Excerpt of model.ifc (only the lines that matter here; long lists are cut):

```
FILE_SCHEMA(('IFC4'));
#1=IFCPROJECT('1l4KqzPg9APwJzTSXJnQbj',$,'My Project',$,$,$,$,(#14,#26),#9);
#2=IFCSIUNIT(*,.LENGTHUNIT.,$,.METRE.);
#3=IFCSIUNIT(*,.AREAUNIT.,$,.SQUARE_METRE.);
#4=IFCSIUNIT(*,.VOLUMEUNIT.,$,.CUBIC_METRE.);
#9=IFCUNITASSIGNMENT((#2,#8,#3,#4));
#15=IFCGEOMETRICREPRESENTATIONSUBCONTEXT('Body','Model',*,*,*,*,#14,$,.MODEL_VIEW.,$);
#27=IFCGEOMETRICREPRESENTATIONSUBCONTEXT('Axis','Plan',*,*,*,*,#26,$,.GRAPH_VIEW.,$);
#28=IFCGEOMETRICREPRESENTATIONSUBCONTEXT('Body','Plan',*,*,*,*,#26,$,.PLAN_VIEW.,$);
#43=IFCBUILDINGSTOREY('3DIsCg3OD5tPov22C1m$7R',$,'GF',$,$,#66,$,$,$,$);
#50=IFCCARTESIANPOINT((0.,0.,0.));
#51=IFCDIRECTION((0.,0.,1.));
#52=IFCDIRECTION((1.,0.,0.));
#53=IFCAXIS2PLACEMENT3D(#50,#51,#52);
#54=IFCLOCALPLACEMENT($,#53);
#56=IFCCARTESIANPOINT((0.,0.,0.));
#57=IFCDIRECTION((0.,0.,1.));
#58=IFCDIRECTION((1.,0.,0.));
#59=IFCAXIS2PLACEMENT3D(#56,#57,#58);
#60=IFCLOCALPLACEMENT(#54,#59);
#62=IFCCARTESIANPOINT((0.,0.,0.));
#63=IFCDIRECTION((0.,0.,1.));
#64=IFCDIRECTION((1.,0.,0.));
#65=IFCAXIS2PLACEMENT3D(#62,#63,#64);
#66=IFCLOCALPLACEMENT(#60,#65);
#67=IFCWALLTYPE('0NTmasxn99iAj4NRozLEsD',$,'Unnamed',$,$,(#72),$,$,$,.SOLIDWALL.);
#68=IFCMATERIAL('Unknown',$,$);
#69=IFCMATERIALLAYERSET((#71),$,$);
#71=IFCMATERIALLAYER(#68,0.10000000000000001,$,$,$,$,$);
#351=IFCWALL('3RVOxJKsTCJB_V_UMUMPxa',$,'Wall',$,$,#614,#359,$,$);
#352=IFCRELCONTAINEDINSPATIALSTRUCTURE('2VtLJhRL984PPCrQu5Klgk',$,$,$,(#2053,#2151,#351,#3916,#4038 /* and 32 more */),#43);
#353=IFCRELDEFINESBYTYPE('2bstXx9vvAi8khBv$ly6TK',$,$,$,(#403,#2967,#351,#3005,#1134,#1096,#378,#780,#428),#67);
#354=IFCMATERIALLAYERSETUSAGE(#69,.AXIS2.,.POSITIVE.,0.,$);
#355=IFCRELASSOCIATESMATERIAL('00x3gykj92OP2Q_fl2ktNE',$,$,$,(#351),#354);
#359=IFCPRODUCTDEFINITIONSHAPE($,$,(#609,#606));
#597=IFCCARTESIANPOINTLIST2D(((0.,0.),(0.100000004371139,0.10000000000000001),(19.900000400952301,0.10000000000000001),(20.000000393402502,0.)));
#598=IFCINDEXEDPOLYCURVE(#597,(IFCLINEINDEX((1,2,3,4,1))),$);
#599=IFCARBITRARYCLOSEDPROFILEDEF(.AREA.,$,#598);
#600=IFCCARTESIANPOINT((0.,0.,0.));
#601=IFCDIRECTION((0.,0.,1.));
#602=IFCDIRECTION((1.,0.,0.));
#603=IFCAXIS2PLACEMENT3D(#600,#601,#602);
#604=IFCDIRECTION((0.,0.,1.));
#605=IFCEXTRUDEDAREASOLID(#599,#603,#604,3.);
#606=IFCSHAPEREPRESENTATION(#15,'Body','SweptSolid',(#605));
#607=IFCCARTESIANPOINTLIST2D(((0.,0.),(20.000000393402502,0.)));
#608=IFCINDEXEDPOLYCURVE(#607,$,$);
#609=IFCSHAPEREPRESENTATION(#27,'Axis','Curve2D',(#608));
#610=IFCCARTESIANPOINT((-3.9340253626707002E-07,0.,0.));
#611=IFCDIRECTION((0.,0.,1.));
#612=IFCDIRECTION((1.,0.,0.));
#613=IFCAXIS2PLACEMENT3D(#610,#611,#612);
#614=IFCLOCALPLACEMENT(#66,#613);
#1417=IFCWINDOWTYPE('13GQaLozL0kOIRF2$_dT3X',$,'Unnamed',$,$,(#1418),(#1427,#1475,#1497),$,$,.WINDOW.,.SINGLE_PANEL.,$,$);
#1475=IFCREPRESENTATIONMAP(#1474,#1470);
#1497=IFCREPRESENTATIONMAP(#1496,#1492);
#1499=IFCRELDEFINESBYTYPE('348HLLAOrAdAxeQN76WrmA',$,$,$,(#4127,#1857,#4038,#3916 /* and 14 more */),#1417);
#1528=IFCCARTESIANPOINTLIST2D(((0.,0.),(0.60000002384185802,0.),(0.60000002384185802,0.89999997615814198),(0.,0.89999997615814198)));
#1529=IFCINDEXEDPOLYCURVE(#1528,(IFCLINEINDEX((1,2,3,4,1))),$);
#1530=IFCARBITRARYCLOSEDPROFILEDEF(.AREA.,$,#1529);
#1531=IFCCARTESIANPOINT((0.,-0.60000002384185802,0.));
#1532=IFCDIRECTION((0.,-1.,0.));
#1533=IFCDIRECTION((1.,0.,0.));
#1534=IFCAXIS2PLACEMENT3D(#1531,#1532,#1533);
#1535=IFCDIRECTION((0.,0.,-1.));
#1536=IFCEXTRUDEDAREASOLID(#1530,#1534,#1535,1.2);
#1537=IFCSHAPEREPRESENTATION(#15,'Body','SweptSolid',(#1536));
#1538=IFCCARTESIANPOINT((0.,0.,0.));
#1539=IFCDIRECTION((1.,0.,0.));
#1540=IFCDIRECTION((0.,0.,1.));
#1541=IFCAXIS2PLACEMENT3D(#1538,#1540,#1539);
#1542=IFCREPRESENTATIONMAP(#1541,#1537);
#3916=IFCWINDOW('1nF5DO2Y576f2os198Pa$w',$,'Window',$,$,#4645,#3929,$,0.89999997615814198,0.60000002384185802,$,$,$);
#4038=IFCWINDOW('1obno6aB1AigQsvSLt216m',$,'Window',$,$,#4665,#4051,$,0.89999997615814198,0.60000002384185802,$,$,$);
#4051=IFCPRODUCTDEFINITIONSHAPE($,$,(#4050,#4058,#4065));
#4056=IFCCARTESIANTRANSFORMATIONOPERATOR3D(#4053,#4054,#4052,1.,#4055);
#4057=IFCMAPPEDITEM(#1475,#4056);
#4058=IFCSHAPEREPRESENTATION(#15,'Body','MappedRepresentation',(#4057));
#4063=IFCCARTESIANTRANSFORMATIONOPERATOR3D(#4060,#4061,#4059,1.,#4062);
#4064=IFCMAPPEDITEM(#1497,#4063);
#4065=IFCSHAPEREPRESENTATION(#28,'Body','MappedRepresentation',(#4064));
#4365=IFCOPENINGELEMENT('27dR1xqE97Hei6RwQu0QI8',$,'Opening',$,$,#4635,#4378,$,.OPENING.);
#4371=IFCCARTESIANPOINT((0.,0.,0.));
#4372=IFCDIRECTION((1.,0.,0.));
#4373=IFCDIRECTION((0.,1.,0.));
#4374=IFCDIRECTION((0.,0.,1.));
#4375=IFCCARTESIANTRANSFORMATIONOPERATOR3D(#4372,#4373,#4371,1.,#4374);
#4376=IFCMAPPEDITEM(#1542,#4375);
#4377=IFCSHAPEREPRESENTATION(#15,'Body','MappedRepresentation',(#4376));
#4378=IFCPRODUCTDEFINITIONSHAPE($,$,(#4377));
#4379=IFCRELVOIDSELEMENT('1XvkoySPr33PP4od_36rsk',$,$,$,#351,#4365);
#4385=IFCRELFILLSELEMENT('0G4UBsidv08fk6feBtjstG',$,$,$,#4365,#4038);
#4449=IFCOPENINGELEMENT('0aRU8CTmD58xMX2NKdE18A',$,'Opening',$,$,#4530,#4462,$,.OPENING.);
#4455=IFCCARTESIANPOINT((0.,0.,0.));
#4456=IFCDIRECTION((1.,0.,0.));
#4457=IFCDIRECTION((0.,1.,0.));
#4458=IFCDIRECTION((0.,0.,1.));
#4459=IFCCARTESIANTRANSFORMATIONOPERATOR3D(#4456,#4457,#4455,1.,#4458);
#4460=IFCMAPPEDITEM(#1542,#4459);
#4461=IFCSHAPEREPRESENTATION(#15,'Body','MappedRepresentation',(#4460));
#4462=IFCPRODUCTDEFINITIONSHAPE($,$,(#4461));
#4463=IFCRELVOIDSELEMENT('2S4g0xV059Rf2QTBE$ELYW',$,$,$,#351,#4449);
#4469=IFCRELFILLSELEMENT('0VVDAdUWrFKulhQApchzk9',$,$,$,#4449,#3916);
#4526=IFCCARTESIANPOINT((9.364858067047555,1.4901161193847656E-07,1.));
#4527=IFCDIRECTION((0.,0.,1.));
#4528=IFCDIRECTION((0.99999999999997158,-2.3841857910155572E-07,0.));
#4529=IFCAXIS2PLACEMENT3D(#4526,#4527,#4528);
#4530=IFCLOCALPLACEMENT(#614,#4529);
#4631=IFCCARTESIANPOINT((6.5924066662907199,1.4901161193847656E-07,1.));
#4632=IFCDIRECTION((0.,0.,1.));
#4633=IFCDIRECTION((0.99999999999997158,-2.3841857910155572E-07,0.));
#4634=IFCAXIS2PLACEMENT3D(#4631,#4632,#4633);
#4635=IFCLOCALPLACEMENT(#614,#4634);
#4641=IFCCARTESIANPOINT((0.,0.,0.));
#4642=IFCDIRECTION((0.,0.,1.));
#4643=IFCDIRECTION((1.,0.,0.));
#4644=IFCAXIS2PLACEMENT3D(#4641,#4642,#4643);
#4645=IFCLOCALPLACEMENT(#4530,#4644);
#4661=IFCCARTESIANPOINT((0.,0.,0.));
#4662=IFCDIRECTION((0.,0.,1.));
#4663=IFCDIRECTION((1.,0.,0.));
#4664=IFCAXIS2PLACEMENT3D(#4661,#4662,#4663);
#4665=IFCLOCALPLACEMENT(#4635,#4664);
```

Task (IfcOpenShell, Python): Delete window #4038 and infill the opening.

```python
import ifcopenshell
import ifcopenshell.api.feature
import ifcopenshell.api.root
import ifcopenshell.geom
import ifcopenshell.util.shape

model = ifcopenshell.open("model.ifc")
settings = ifcopenshell.geom.settings()


def volume(element):
    """Net volume in cubic metres, openings subtracted."""
    shape = ifcopenshell.geom.create_shape(settings, element)
    return ifcopenshell.util.shape.get_volume(shape.geometry)


window = model.by_guid("1obno6aB1AigQsvSLt216m")
opening = window.FillsVoids[0].RelatingOpeningElement
wall = opening.VoidsElements[0].RelatingBuildingElement
before = volume(wall)

ifcopenshell.api.root.remove_product(model, product=window)
ifcopenshell.api.feature.remove_feature(model, feature=opening)

after = volume(wall)

print(f"wall volume {before:.3f} -> {after:.3f} m3")

model.write("model_edited.ifc")
```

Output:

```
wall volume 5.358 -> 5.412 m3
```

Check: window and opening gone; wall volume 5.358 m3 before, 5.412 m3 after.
